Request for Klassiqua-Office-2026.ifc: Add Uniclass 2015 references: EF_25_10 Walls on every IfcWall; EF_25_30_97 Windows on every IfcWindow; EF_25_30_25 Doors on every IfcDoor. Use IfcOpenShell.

First a look at what the model holds.

```python
import ifcopenshell

model = ifcopenshell.open("Klassiqua-Office-2026.ifc")
print(model.schema)
print("classifications:", [c.Name for c in model.by_type("IfcClassification")])
for ifc_class in ("IfcDoor", "IfcRoof", "IfcStair", "IfcWall", "IfcWindow"):
    print(ifc_class, len(model.by_type(ifc_class)))
```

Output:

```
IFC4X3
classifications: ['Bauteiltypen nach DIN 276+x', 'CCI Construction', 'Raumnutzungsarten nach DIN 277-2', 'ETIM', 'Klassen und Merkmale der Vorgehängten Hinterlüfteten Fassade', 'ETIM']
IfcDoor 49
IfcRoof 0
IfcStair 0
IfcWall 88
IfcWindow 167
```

```python
import ifcopenshell
import ifcopenshell.api.classification

model = ifcopenshell.open("Klassiqua-Office-2026.ifc")

system = ifcopenshell.api.classification.add_classification(model, classification="Uniclass 2015")

codes = {
    "IfcWall": ("EF_25_10", "Walls"),
    "IfcWindow": ("EF_25_30_97", "Windows"),
    "IfcDoor": ("EF_25_30_25", "Doors"),
}
for ifc_class, (code, name) in codes.items():
    products = model.by_type(ifc_class)
    ifcopenshell.api.classification.add_reference(
        model, products=products, classification=system, identification=code, name=name
    )
    print(code, len(products))

model.write("Klassiqua-Office-2026_edited.ifc")
```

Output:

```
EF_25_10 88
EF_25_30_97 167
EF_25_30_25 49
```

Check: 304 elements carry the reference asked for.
